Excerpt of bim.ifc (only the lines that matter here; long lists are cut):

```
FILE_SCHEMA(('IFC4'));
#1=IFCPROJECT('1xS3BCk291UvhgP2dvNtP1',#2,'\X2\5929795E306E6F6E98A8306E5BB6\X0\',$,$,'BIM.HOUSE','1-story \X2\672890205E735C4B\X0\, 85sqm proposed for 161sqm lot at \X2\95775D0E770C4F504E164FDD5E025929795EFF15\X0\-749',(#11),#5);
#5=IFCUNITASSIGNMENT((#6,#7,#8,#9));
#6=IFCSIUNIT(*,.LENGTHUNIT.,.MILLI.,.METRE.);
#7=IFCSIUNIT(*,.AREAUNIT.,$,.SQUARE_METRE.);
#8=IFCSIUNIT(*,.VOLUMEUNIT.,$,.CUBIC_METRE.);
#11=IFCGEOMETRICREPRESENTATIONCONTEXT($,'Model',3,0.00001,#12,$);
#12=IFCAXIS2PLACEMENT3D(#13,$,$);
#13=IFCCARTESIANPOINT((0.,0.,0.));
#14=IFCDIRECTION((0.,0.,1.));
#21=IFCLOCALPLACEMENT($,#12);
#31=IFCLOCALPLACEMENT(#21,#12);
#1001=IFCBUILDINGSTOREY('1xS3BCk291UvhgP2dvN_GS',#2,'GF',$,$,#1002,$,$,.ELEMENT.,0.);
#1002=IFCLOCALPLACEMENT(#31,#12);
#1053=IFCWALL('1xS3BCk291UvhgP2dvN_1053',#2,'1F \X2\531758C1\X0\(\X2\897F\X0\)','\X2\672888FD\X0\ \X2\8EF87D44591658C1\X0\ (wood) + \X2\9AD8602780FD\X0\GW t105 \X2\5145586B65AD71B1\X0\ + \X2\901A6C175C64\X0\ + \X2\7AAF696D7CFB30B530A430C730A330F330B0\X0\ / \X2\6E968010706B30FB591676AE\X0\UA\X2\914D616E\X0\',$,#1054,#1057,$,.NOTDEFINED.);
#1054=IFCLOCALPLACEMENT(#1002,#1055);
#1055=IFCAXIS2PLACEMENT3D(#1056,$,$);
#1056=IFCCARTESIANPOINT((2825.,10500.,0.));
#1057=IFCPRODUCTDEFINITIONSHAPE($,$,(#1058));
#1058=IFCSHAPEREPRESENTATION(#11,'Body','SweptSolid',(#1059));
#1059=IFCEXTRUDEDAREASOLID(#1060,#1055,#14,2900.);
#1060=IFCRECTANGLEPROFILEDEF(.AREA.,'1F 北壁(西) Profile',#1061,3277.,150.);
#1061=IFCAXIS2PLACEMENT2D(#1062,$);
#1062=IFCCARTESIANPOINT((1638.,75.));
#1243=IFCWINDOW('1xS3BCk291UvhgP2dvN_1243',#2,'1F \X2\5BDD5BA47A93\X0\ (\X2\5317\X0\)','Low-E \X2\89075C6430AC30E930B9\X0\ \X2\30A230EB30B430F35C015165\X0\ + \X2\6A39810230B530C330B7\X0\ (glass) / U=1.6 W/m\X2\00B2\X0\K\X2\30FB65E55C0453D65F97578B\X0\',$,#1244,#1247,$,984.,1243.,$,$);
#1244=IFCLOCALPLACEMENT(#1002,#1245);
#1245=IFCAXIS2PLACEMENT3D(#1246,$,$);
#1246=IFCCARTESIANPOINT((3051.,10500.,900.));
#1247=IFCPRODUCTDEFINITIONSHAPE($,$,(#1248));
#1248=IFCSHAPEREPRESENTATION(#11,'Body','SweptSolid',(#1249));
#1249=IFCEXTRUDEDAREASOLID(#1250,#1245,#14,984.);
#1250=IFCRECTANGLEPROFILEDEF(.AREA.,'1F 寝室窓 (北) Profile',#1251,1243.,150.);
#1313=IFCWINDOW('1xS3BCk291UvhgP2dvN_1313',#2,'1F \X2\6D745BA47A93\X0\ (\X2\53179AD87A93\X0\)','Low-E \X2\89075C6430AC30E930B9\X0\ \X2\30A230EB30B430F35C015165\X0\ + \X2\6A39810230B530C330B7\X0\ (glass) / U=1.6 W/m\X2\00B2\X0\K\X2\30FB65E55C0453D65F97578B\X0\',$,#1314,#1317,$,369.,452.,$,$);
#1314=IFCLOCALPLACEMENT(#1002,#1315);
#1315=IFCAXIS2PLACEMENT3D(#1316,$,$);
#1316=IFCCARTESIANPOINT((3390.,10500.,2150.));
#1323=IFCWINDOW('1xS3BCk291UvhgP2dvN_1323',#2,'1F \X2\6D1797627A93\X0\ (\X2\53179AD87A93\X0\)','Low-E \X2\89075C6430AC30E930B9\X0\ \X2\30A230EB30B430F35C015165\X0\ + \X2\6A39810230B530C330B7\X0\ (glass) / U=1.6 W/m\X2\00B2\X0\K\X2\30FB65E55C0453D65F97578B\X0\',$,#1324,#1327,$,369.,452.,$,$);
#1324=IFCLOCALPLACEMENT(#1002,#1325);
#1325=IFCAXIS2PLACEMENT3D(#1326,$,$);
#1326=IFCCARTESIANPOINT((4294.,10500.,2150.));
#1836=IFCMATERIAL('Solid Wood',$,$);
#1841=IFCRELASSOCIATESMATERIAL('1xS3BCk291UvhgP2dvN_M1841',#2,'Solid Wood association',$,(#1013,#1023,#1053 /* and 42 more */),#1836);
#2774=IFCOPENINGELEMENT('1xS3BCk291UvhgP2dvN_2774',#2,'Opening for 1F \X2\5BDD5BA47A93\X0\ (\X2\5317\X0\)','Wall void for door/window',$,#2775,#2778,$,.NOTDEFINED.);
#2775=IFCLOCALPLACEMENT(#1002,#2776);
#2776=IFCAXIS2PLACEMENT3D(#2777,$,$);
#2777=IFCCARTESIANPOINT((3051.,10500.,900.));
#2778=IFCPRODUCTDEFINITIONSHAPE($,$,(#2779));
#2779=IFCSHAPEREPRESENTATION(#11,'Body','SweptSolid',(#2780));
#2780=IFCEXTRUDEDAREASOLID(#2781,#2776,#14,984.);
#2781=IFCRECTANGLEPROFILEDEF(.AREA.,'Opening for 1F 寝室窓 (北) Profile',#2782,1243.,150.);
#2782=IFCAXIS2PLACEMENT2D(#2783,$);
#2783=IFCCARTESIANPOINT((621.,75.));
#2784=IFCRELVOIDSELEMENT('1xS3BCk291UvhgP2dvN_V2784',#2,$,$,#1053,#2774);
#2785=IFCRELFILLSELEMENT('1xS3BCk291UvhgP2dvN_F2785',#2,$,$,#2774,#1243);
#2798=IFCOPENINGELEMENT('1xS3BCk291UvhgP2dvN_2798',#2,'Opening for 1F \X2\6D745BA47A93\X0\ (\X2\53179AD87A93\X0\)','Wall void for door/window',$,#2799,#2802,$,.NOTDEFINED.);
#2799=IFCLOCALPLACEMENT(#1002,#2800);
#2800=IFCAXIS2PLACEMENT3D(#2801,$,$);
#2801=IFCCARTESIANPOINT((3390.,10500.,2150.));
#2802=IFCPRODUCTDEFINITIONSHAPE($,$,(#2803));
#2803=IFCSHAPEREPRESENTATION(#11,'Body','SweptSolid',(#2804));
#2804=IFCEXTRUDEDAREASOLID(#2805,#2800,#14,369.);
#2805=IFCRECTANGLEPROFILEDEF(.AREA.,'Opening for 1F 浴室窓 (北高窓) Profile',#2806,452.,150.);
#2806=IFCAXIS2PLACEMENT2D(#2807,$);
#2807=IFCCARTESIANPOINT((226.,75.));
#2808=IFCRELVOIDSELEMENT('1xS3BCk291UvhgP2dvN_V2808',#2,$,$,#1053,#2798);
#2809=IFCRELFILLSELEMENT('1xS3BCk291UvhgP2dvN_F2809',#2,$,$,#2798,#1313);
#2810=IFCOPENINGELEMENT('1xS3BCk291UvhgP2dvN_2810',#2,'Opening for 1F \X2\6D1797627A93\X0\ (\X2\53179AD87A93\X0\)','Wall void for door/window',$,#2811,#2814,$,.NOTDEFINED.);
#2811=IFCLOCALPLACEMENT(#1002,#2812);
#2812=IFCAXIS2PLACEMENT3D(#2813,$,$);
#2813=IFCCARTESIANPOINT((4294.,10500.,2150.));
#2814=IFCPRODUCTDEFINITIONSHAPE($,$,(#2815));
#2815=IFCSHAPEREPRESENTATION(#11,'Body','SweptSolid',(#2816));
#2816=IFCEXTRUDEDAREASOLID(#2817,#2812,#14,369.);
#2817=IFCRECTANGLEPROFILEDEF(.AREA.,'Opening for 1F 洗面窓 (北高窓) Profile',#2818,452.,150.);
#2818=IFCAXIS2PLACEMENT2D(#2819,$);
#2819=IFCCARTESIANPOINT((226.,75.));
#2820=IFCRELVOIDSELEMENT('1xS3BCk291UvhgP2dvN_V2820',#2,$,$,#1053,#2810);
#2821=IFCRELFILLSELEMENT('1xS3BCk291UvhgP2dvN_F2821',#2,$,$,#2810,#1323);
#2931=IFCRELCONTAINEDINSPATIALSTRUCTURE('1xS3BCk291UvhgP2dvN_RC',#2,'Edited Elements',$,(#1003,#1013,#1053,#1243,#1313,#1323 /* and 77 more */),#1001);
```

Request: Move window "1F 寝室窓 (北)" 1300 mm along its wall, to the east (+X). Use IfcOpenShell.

```python
import ifcopenshell
import ifcopenshell.api.geometry
import ifcopenshell.util.placement

model = ifcopenshell.open("bim.ifc")

window = model.by_guid("1xS3BCk291UvhgP2dvN_1243")
opening = window.FillsVoids[0].RelatingOpeningElement
wall = opening.VoidsElements[0].RelatingBuildingElement

wall_matrix = ifcopenshell.util.placement.get_local_placement(wall.ObjectPlacement)
shift = wall_matrix[:3, 0] * 1300.0
before = ifcopenshell.util.placement.get_local_placement(window.ObjectPlacement)[:3, 3].copy()

# The window is not placed relative to its opening, so move both.
for product in (opening, window):
    matrix = ifcopenshell.util.placement.get_local_placement(product.ObjectPlacement)
    matrix[:3, 3] += shift
    ifcopenshell.api.geometry.edit_object_placement(model, product=product, matrix=matrix, is_si=False)

after = ifcopenshell.util.placement.get_local_placement(window.ObjectPlacement)[:3, 3]
print("window moved by", (after - before).round(3) + 0.0)

model.write("bim-out.ifc")
```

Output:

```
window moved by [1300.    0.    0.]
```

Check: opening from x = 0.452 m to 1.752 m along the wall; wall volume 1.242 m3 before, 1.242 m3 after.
